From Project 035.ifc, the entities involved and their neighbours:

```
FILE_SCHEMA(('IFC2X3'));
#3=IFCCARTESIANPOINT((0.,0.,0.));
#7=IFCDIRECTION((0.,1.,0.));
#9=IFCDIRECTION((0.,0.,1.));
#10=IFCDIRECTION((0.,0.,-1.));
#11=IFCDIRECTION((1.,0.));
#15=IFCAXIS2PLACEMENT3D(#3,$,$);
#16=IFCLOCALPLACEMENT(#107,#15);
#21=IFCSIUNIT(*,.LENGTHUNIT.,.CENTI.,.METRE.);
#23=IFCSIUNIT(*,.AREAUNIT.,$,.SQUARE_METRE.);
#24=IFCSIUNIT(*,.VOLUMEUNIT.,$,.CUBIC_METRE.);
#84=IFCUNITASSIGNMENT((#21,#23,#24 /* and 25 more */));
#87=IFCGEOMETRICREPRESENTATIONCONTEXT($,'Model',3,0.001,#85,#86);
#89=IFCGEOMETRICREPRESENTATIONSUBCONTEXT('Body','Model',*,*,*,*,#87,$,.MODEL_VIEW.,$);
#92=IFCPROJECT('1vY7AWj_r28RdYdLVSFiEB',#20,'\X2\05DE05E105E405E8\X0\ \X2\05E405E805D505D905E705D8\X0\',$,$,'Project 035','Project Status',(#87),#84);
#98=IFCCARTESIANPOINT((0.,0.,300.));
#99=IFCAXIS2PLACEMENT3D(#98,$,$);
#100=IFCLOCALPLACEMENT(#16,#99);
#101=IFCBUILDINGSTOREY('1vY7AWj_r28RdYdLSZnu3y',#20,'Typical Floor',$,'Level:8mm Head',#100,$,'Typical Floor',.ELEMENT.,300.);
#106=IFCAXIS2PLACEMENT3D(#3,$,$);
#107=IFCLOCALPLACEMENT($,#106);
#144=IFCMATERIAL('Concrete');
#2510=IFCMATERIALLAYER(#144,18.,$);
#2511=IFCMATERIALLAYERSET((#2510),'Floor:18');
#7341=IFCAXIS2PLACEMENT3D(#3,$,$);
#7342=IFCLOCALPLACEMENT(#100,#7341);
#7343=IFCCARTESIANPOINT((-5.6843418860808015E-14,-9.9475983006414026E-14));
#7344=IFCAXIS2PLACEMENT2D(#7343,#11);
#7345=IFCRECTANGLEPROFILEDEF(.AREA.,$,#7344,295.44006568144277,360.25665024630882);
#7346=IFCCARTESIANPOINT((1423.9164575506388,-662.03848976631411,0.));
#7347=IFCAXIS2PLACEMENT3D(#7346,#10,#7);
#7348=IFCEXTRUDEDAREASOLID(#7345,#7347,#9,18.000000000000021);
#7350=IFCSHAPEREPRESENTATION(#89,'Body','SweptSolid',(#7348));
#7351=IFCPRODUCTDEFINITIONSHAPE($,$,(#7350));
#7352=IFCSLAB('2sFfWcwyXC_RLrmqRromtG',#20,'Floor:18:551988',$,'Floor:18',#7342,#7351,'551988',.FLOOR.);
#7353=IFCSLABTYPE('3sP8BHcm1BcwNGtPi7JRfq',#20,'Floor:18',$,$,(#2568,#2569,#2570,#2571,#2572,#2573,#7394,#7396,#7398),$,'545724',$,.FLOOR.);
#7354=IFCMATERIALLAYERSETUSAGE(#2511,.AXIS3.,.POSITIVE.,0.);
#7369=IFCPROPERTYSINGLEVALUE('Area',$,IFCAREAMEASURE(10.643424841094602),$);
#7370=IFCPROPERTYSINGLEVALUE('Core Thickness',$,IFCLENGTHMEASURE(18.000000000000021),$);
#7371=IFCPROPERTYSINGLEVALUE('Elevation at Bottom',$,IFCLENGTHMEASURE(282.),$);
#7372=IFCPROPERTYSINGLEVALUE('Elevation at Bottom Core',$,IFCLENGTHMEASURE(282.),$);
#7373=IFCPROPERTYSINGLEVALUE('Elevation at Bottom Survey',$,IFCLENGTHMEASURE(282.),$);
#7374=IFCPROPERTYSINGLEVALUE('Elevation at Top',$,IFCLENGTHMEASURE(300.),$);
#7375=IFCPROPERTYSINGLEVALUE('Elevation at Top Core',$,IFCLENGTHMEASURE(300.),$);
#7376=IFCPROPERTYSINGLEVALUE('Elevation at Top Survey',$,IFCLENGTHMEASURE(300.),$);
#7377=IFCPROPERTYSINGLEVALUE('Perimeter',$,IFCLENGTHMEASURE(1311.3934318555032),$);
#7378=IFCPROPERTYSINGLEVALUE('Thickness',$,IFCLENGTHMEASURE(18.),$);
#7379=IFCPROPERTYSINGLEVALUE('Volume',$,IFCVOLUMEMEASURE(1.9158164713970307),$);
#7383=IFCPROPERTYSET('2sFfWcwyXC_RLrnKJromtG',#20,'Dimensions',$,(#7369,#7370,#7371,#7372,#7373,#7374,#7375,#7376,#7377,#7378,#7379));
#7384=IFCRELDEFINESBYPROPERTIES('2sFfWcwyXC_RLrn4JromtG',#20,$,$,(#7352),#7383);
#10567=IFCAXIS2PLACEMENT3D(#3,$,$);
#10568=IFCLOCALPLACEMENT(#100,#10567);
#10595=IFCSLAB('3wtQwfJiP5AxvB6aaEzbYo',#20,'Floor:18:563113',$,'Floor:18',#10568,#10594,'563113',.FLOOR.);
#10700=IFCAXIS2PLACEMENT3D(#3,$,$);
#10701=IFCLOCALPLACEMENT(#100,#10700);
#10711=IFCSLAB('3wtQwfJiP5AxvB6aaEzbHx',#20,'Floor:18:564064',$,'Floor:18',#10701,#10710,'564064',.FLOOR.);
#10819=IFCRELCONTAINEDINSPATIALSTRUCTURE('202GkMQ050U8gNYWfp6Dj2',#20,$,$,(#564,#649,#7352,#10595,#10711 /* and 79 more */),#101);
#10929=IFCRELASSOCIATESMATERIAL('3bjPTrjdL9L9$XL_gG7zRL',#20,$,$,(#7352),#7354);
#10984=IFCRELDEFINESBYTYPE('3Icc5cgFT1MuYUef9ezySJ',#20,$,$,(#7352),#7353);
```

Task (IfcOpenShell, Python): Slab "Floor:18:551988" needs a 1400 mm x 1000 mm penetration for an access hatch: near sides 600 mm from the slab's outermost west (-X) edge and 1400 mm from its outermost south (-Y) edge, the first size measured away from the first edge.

```python
import numpy as np
import ifcopenshell
import ifcopenshell.api.feature
import ifcopenshell.api.geometry
import ifcopenshell.api.pset
import ifcopenshell.api.root
import ifcopenshell.geom
import ifcopenshell.util.element
import ifcopenshell.util.placement
import ifcopenshell.util.representation
import ifcopenshell.util.shape
import ifcopenshell.util.unit

model = ifcopenshell.open("Project 035.ifc")
unit_scale = ifcopenshell.util.unit.calculate_unit_scale(model)
area_scale = ifcopenshell.util.unit.calculate_unit_scale(model, "AREAUNIT")
volume_scale = ifcopenshell.util.unit.calculate_unit_scale(model, "VOLUMEUNIT")
settings = ifcopenshell.geom.settings()


def volume(element):
    """Net volume in cubic metres, openings subtracted."""
    shape = ifcopenshell.geom.create_shape(settings, element)
    return ifcopenshell.util.shape.get_volume(shape.geometry)


slab = model.by_guid("2sFfWcwyXC_RLrmqRromtG")
before = volume(slab)

# Extent in the slab's own axes, in metres. The edges named are its -X and -Y sides.
slab_shape = ifcopenshell.geom.create_shape(settings, slab)
vertices = ifcopenshell.util.shape.get_vertices(slab_shape.geometry)
x_min, y_min, bottom = vertices.min(axis=0)
top = vertices[:, 2].max()

opening = ifcopenshell.api.root.create_entity(model, ifc_class="IfcOpeningElement", name="Access hatch opening")
context = ifcopenshell.util.representation.get_context(model, "Model", "Body", "MODEL_VIEW")
width, depth = 1.4, 1
outline = [(0.0, 0.0), (width, 0.0), (width, depth), (0.0, depth), (0.0, 0.0)]
# Overshoot both faces by 50 mm so the cut is clean.
shape = ifcopenshell.api.geometry.add_slab_representation(
    model, context=context, depth=top - bottom + 0.1, polyline=outline
)
ifcopenshell.api.geometry.assign_representation(model, product=opening, representation=shape)

matrix = ifcopenshell.util.placement.get_local_placement(slab.ObjectPlacement)
matrix[:, 3] = matrix @ np.append(np.array([x_min + 0.6, y_min + 1.4, bottom - 0.05]) / unit_scale, 1.0)
ifcopenshell.api.geometry.edit_object_placement(model, product=opening, matrix=matrix, is_si=False)
ifcopenshell.api.feature.add_feature(model, feature=opening, element=slab)

after = volume(slab)

# Update the slab's stored quantities.
pset = model.by_id(ifcopenshell.util.element.get_pset(slab, "Dimensions", should_inherit=False)["id"])
ifcopenshell.api.pset.edit_pset(model, pset=pset, properties={
    "Area": model.create_entity("IfcAreaMeasure", after / (top - bottom) / area_scale),
    "Volume": model.create_entity("IfcVolumeMeasure", after / volume_scale),
})

print(f"slab volume {before:.3f} -> {after:.3f} m3")

model.write("Project 035_v2.ifc")
```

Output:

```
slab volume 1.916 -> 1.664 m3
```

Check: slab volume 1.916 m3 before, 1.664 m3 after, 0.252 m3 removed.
